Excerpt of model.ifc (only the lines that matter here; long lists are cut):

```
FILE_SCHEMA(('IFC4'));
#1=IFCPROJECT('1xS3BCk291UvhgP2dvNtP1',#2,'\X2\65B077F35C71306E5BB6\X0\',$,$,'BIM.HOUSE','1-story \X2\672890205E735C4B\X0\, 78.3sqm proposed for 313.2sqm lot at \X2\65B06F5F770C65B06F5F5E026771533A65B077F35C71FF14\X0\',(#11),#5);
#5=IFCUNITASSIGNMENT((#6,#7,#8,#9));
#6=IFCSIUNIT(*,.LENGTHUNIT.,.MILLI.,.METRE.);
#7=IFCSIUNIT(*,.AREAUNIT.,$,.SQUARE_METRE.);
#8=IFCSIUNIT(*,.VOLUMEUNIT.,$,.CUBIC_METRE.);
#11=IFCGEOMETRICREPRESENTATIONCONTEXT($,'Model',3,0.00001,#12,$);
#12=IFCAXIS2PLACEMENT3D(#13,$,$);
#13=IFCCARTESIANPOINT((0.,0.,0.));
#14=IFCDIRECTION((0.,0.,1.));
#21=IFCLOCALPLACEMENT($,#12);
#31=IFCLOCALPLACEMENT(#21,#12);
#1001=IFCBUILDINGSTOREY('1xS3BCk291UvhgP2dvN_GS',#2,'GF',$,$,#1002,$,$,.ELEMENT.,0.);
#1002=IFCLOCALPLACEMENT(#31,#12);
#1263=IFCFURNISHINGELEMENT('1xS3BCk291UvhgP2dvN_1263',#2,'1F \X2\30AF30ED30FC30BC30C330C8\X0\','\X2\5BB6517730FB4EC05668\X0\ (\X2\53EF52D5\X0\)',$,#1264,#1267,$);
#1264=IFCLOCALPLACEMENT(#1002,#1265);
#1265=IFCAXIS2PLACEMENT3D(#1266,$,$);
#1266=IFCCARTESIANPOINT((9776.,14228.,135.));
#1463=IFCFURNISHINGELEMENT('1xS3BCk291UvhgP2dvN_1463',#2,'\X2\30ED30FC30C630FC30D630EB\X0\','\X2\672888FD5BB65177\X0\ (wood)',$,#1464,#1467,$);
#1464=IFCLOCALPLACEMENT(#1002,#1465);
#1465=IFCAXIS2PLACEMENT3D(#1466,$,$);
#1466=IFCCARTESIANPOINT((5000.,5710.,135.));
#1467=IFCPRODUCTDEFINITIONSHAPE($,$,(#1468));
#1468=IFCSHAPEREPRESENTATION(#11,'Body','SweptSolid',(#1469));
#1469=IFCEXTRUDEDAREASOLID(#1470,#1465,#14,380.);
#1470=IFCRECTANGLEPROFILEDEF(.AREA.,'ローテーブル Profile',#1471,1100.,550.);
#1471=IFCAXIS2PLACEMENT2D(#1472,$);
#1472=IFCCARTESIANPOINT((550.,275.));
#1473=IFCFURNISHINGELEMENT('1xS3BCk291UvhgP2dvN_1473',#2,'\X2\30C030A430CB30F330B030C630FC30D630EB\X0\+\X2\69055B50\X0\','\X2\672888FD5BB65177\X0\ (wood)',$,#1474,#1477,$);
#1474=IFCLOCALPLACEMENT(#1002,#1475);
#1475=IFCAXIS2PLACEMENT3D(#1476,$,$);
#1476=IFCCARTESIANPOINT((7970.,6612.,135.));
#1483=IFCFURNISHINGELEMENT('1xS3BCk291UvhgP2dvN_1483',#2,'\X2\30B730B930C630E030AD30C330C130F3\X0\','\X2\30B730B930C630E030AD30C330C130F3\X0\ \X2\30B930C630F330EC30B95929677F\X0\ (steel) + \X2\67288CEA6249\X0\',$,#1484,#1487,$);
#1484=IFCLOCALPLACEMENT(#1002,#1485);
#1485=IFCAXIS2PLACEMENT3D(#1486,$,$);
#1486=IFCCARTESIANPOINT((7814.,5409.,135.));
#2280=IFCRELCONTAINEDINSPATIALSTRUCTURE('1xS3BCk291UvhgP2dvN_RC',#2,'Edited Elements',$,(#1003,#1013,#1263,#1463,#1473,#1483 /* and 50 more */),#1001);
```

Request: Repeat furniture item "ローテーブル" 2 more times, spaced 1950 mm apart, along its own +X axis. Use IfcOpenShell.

```python
import ifcopenshell
import ifcopenshell.api.geometry
import ifcopenshell.api.root
import ifcopenshell.util.element
import ifcopenshell.util.placement
import ifcopenshell.util.unit

model = ifcopenshell.open("model.ifc")
unit_scale = ifcopenshell.util.unit.calculate_unit_scale(model)


def reuse_history(source, copy):
    """copy_class also copies each property set's owner history, people and application; keep the originals."""
    for rel in copy.IsDefinedBy:
        if rel.is_a("IfcRelDefinesByProperties") and (history := rel.RelatingPropertyDefinition.OwnerHistory):
            rel.RelatingPropertyDefinition.OwnerHistory = source.OwnerHistory
            ifcopenshell.util.element.remove_deep2(model, history)


source = model.by_guid("1xS3BCk291UvhgP2dvN_1463")
base = ifcopenshell.util.placement.get_local_placement(source.ObjectPlacement)
step = base[:3, 0] * 1.95 / unit_scale

for i in range(1, 3):
    copy = ifcopenshell.api.root.copy_class(model, product=source)
    copy.Representation = ifcopenshell.util.element.copy_deep(
        model, source.Representation, exclude=["IfcGeometricRepresentationContext", "IfcRepresentationMap"]
    )
    reuse_history(source, copy)
    matrix = base.copy()
    matrix[:3, 3] += i * step
    print("added at", matrix[:3, 3].round(3) + 0.0)
    ifcopenshell.api.geometry.edit_object_placement(model, product=copy, matrix=matrix, is_si=False)

model.write("model_edited.ifc")
```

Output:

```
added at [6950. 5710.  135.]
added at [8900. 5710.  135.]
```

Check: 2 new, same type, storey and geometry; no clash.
